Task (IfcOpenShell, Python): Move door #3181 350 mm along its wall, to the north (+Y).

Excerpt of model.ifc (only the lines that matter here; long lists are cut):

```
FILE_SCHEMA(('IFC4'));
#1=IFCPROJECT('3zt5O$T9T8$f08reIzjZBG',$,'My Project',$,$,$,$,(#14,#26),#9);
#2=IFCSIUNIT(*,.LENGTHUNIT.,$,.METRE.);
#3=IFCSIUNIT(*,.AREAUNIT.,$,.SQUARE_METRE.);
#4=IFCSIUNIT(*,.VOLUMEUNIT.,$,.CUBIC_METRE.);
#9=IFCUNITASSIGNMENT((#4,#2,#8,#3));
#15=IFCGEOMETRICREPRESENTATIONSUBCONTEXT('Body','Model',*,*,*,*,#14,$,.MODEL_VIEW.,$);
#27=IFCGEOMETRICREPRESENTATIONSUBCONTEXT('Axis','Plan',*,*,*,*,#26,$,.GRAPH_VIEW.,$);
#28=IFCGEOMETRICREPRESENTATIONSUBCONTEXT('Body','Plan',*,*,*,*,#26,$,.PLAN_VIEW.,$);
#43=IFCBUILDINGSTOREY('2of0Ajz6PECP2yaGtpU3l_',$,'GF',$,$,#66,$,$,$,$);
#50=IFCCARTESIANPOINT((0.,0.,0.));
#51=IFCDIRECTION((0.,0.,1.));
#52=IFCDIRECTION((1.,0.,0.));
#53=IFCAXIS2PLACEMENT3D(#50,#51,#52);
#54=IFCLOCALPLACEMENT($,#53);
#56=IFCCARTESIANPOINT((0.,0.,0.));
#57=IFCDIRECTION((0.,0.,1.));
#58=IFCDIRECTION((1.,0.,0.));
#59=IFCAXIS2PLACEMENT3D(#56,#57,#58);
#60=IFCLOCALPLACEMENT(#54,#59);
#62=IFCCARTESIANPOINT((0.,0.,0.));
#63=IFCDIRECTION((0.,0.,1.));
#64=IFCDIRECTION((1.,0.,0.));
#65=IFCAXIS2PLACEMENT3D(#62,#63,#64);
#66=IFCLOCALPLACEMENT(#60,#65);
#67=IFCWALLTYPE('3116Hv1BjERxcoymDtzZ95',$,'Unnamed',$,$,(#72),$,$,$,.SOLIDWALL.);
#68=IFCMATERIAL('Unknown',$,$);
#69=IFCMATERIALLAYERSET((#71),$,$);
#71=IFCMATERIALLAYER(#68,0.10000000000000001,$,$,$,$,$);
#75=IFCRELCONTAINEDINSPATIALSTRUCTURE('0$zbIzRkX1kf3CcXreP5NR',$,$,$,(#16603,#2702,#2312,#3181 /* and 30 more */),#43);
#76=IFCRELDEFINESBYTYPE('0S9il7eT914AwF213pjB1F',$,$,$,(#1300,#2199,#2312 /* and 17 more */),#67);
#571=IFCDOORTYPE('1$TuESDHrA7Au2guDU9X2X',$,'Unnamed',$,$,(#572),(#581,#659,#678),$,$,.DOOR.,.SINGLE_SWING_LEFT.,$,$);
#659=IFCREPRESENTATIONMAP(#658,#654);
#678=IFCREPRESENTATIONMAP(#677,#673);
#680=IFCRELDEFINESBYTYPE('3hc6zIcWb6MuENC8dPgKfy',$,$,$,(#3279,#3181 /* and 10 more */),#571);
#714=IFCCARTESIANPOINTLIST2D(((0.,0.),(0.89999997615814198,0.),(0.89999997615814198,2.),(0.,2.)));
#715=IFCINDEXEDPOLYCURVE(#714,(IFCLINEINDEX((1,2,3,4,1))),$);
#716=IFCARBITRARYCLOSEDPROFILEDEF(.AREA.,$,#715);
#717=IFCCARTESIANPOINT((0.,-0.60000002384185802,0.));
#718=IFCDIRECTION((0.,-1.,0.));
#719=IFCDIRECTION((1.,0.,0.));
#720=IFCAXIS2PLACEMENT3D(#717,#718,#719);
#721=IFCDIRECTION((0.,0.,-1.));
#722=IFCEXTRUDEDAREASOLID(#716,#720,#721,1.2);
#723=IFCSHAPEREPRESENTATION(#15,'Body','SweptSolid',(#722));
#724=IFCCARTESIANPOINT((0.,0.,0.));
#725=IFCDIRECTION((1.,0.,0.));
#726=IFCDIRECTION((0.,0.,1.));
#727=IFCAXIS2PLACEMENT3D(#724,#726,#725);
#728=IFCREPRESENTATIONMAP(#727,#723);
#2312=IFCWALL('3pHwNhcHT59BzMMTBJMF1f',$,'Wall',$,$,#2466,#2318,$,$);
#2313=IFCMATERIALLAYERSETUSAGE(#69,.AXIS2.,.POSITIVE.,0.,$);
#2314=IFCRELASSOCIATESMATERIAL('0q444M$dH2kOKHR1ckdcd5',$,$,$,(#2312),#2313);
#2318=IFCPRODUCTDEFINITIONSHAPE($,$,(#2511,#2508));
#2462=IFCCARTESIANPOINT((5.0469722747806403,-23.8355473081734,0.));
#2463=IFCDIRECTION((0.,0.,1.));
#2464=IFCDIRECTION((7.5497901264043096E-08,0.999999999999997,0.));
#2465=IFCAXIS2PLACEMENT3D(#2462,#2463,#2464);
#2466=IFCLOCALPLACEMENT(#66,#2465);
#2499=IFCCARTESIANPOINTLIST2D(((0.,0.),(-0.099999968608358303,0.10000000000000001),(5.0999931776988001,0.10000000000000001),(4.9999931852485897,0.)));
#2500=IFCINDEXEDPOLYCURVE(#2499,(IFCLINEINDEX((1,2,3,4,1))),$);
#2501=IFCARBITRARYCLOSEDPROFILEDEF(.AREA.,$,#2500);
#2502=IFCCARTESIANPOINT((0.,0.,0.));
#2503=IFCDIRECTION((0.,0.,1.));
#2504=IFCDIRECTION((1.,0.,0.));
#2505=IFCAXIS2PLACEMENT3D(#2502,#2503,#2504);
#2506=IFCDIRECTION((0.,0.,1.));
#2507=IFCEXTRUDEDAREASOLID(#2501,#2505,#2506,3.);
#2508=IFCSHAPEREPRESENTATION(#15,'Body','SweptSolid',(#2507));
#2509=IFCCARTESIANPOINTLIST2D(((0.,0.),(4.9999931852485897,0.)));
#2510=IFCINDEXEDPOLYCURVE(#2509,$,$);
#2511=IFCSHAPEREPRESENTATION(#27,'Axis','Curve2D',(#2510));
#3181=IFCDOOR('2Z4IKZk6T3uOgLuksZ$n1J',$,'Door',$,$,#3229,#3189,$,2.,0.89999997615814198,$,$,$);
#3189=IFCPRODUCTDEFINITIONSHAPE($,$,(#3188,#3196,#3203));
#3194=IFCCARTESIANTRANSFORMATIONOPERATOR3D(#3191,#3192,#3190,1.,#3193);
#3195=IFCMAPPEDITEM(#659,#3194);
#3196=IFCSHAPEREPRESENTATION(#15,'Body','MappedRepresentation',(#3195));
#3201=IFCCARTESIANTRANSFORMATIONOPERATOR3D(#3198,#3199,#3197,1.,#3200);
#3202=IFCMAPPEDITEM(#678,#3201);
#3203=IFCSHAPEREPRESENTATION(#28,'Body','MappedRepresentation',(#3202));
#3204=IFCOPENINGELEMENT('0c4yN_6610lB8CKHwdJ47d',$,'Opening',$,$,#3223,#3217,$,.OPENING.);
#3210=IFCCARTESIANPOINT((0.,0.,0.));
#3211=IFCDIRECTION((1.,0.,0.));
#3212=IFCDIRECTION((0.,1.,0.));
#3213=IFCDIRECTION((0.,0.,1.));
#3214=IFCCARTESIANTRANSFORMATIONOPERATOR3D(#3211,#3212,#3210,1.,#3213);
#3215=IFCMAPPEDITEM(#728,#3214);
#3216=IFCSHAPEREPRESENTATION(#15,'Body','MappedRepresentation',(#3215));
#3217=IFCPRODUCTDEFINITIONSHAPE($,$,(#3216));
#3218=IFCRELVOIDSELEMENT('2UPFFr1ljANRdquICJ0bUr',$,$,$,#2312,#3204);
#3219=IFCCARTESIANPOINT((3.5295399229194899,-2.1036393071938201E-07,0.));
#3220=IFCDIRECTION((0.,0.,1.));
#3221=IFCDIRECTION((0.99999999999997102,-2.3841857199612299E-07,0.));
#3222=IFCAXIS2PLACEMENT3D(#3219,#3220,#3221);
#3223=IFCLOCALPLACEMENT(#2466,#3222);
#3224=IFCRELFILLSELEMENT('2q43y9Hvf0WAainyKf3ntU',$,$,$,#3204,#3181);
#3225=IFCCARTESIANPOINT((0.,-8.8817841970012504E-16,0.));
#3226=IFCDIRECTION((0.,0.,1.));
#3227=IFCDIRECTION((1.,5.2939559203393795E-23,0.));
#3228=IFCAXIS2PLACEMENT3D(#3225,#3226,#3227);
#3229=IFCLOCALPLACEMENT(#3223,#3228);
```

```python
import ifcopenshell
import ifcopenshell.api.geometry
import ifcopenshell.util.placement
import ifcopenshell.util.unit

model = ifcopenshell.open("model.ifc")
unit_scale = ifcopenshell.util.unit.calculate_unit_scale(model)

door = model.by_guid("2Z4IKZk6T3uOgLuksZ$n1J")
opening = door.FillsVoids[0].RelatingOpeningElement
wall = opening.VoidsElements[0].RelatingBuildingElement

wall_matrix = ifcopenshell.util.placement.get_local_placement(wall.ObjectPlacement)
shift = wall_matrix[:3, 0] * 0.35 / unit_scale
before = ifcopenshell.util.placement.get_local_placement(door.ObjectPlacement)[:3, 3].copy()

# The door is placed relative to its opening, so it follows when the opening moves.
matrix = ifcopenshell.util.placement.get_local_placement(opening.ObjectPlacement)
matrix[:3, 3] += shift
ifcopenshell.api.geometry.edit_object_placement(
    model, product=opening, matrix=matrix, is_si=False, should_transform_children=True
)

after = ifcopenshell.util.placement.get_local_placement(door.ObjectPlacement)[:3, 3]
print("door moved by", (after - before).round(3) + 0.0)

model.write("model_edited.ifc")
```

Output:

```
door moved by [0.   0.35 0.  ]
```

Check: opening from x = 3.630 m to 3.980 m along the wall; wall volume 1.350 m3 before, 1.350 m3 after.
